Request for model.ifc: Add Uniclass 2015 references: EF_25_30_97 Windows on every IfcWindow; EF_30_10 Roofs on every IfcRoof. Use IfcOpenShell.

First a look at what the model holds.

```python
import ifcopenshell

model = ifcopenshell.open("model.ifc")
print(model.schema)
print("classifications:", [c.Name for c in model.by_type("IfcClassification")])
for ifc_class in ("IfcDoor", "IfcRoof", "IfcStair", "IfcWall", "IfcWindow"):
    print(ifc_class, len(model.by_type(ifc_class)))
```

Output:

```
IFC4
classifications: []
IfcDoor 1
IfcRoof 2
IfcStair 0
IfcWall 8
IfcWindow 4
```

```python
import ifcopenshell
import ifcopenshell.api.classification

model = ifcopenshell.open("model.ifc")

system = ifcopenshell.api.classification.add_classification(model, classification="Uniclass 2015")

codes = {
    "IfcWindow": ("EF_25_30_97", "Windows"),
    "IfcRoof": ("EF_30_10", "Roofs"),
}
for ifc_class, (code, name) in codes.items():
    products = model.by_type(ifc_class)
    ifcopenshell.api.classification.add_reference(
        model, products=products, classification=system, identification=code, name=name
    )
    print(code, len(products))

model.write("model_edited.ifc")
```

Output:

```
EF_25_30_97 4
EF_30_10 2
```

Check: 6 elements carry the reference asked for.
